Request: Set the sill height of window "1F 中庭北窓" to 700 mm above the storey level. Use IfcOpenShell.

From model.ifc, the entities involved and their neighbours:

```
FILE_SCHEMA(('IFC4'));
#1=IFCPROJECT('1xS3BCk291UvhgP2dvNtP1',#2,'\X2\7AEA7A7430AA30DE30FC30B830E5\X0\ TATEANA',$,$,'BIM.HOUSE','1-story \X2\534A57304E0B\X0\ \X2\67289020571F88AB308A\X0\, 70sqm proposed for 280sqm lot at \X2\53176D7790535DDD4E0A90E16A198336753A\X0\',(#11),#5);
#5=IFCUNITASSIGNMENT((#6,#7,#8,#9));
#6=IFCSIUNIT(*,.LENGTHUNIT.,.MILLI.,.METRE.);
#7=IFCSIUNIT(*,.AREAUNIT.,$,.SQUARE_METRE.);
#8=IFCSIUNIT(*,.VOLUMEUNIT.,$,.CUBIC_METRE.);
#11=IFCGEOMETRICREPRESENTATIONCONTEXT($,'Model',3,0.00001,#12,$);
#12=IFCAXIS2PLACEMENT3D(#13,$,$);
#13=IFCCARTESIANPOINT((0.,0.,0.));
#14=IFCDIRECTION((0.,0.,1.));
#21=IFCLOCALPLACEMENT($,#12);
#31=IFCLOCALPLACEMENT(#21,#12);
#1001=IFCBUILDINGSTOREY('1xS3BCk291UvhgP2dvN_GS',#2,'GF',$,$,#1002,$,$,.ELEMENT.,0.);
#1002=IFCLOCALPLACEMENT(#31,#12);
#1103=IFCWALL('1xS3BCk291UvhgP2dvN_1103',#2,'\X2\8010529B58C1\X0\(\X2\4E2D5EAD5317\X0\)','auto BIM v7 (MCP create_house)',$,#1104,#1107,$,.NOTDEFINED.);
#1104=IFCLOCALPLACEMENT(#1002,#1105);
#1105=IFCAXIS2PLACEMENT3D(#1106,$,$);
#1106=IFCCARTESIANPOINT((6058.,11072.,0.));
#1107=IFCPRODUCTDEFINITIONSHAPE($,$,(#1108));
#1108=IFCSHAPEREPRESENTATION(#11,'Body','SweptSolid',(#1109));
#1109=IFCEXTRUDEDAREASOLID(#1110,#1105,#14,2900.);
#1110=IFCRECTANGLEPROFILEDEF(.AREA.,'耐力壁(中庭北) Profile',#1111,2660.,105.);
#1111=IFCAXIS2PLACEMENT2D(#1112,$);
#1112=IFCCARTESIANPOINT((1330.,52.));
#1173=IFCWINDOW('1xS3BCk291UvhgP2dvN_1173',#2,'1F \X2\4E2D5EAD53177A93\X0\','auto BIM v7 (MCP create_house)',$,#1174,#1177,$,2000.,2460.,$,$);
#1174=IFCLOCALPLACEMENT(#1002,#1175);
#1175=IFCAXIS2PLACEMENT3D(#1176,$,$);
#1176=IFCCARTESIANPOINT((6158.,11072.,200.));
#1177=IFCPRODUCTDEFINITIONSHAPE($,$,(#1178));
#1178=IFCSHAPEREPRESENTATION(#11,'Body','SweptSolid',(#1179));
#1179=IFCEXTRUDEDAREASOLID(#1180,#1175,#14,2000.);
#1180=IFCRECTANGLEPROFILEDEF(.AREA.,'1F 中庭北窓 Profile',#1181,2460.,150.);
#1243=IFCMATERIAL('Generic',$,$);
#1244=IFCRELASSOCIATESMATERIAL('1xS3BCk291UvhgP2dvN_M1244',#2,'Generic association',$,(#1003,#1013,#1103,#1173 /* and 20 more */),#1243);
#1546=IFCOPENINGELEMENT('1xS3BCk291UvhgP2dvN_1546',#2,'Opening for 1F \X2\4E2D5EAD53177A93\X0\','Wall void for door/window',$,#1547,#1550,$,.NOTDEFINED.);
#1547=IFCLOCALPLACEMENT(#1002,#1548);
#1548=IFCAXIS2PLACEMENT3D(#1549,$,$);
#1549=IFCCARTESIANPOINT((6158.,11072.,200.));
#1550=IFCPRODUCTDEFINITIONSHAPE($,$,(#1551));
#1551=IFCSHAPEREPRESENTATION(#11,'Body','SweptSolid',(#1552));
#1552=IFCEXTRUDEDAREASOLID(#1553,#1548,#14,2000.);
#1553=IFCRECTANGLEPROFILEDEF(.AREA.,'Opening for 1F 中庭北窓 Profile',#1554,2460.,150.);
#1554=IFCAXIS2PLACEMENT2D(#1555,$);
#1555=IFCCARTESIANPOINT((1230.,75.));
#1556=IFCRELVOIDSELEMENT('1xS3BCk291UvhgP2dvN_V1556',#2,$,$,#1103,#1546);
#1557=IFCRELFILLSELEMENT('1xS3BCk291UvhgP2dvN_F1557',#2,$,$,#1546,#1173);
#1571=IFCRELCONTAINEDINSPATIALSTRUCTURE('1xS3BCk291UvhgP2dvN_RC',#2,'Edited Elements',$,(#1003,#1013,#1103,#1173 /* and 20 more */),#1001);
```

```python
import numpy as np
import ifcopenshell
import ifcopenshell.api.geometry
import ifcopenshell.geom
import ifcopenshell.util.element
import ifcopenshell.util.placement
import ifcopenshell.util.shape
import ifcopenshell.util.unit

model = ifcopenshell.open("model.ifc")
unit_scale = ifcopenshell.util.unit.calculate_unit_scale(model)

window = model.by_guid("1xS3BCk291UvhgP2dvN_1173")
opening = window.FillsVoids[0].RelatingOpeningElement
storey = ifcopenshell.util.element.get_container(window, ifc_class="IfcBuildingStorey")
level = ifcopenshell.util.placement.get_local_placement(storey.ObjectPlacement)[2, 3]

# The opening's origin need not be at the sill, so measure its lowest point.
shape = ifcopenshell.geom.create_shape(ifcopenshell.geom.settings(), opening)
bottom = ifcopenshell.util.shape.get_shape_bottom_elevation(shape, shape.geometry) / unit_scale
dz = level + 0.7 / unit_scale - bottom

shift = np.array([0.0, 0.0, dz])
# The window is not placed relative to its opening, so move both.
for product in (opening, window):
    matrix = ifcopenshell.util.placement.get_local_placement(product.ObjectPlacement)
    matrix[:3, 3] += shift
    ifcopenshell.api.geometry.edit_object_placement(model, product=product, matrix=matrix, is_si=False)

print(f"moved by {dz * unit_scale:+.3f} m")

model.write("model_updated.ifc")
```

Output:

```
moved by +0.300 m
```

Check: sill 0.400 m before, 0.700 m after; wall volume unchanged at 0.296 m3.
